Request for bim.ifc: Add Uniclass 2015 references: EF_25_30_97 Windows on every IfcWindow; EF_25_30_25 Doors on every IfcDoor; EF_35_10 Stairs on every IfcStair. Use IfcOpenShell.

First a look at what the model holds.

```python
import ifcopenshell

model = ifcopenshell.open("bim.ifc")
print(model.schema)
print("classifications:", [c.Name for c in model.by_type("IfcClassification")])
for ifc_class in ("IfcDoor", "IfcRoof", "IfcStair", "IfcWall", "IfcWindow"):
    print(ifc_class, len(model.by_type(ifc_class)))
```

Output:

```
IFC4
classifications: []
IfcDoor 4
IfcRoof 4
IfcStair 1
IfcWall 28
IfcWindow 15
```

```python
import ifcopenshell
import ifcopenshell.api.classification

model = ifcopenshell.open("bim.ifc")

system = ifcopenshell.api.classification.add_classification(model, classification="Uniclass 2015")

codes = {
    "IfcWindow": ("EF_25_30_97", "Windows"),
    "IfcDoor": ("EF_25_30_25", "Doors"),
    "IfcStair": ("EF_35_10", "Stairs"),
}
for ifc_class, (code, name) in codes.items():
    products = model.by_type(ifc_class)
    ifcopenshell.api.classification.add_reference(
        model, products=products, classification=system, identification=code, name=name
    )
    print(code, len(products))

model.write("bim_edited.ifc")
```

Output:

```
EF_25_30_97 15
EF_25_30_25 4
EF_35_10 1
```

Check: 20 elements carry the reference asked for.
